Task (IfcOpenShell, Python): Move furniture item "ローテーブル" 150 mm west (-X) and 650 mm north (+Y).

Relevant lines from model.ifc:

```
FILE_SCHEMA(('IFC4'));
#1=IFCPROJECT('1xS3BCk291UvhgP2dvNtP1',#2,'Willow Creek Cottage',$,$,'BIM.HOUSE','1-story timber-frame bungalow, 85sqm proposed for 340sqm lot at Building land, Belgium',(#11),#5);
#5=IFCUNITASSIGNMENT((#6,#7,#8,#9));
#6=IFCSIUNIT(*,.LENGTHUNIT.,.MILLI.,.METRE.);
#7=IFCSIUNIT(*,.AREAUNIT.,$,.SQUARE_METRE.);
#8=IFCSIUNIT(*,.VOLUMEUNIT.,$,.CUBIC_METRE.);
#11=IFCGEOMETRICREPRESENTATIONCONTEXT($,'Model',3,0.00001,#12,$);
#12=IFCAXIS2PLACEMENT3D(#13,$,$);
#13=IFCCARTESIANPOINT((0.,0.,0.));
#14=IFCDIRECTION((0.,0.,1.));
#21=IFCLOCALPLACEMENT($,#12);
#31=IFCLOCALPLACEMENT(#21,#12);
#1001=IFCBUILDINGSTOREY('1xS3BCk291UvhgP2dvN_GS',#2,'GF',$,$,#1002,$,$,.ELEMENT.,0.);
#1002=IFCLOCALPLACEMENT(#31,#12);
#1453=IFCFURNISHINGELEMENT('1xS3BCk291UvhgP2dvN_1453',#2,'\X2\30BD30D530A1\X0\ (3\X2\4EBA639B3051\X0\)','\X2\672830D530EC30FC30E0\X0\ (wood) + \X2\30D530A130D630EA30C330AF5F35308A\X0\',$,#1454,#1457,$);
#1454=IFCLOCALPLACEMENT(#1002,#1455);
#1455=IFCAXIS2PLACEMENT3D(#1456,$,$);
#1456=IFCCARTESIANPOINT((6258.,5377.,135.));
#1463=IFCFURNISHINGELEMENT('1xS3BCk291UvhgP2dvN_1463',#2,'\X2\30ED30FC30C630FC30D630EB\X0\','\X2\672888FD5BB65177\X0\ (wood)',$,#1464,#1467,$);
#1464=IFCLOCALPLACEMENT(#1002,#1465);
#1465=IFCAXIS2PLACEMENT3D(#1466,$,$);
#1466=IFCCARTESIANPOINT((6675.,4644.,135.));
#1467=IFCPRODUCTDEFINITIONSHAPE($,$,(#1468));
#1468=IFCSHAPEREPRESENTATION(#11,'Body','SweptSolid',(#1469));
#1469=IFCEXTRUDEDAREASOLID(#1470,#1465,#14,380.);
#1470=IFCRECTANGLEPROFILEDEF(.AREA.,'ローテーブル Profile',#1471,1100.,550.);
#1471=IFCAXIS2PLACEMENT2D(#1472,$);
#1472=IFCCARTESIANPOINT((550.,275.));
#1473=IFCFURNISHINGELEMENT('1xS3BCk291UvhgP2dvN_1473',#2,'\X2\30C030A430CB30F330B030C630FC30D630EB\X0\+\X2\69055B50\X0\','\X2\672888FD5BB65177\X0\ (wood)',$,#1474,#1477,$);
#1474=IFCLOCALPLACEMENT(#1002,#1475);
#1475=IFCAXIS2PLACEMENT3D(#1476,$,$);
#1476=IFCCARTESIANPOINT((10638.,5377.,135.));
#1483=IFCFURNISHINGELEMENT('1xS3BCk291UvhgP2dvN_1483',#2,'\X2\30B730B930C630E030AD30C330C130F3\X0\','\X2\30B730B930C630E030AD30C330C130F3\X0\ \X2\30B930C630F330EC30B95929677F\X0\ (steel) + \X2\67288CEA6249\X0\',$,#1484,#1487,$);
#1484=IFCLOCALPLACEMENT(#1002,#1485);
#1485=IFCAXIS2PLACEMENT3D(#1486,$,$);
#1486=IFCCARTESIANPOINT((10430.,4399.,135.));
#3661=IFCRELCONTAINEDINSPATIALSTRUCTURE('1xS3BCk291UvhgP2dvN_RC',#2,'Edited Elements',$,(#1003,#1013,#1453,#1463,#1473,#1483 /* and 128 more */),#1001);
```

```python
import ifcopenshell
import ifcopenshell.api.geometry
import ifcopenshell.util.placement
import ifcopenshell.util.unit

model = ifcopenshell.open("model.ifc")
unit_scale = ifcopenshell.util.unit.calculate_unit_scale(model)

item = model.by_guid("1xS3BCk291UvhgP2dvN_1463")
matrix = ifcopenshell.util.placement.get_local_placement(item.ObjectPlacement)
matrix[0, 3] -= 0.15 / unit_scale
matrix[1, 3] += 0.65 / unit_scale
ifcopenshell.api.geometry.edit_object_placement(model, product=item, matrix=matrix, is_si=False)

print(ifcopenshell.util.placement.get_local_placement(item.ObjectPlacement).round(3) + 0.0)

model.write("model_updated.ifc")
```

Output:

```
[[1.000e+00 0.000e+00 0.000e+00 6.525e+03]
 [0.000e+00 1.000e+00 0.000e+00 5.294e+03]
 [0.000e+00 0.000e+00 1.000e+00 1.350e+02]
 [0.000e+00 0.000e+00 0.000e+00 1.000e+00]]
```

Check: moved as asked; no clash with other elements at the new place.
